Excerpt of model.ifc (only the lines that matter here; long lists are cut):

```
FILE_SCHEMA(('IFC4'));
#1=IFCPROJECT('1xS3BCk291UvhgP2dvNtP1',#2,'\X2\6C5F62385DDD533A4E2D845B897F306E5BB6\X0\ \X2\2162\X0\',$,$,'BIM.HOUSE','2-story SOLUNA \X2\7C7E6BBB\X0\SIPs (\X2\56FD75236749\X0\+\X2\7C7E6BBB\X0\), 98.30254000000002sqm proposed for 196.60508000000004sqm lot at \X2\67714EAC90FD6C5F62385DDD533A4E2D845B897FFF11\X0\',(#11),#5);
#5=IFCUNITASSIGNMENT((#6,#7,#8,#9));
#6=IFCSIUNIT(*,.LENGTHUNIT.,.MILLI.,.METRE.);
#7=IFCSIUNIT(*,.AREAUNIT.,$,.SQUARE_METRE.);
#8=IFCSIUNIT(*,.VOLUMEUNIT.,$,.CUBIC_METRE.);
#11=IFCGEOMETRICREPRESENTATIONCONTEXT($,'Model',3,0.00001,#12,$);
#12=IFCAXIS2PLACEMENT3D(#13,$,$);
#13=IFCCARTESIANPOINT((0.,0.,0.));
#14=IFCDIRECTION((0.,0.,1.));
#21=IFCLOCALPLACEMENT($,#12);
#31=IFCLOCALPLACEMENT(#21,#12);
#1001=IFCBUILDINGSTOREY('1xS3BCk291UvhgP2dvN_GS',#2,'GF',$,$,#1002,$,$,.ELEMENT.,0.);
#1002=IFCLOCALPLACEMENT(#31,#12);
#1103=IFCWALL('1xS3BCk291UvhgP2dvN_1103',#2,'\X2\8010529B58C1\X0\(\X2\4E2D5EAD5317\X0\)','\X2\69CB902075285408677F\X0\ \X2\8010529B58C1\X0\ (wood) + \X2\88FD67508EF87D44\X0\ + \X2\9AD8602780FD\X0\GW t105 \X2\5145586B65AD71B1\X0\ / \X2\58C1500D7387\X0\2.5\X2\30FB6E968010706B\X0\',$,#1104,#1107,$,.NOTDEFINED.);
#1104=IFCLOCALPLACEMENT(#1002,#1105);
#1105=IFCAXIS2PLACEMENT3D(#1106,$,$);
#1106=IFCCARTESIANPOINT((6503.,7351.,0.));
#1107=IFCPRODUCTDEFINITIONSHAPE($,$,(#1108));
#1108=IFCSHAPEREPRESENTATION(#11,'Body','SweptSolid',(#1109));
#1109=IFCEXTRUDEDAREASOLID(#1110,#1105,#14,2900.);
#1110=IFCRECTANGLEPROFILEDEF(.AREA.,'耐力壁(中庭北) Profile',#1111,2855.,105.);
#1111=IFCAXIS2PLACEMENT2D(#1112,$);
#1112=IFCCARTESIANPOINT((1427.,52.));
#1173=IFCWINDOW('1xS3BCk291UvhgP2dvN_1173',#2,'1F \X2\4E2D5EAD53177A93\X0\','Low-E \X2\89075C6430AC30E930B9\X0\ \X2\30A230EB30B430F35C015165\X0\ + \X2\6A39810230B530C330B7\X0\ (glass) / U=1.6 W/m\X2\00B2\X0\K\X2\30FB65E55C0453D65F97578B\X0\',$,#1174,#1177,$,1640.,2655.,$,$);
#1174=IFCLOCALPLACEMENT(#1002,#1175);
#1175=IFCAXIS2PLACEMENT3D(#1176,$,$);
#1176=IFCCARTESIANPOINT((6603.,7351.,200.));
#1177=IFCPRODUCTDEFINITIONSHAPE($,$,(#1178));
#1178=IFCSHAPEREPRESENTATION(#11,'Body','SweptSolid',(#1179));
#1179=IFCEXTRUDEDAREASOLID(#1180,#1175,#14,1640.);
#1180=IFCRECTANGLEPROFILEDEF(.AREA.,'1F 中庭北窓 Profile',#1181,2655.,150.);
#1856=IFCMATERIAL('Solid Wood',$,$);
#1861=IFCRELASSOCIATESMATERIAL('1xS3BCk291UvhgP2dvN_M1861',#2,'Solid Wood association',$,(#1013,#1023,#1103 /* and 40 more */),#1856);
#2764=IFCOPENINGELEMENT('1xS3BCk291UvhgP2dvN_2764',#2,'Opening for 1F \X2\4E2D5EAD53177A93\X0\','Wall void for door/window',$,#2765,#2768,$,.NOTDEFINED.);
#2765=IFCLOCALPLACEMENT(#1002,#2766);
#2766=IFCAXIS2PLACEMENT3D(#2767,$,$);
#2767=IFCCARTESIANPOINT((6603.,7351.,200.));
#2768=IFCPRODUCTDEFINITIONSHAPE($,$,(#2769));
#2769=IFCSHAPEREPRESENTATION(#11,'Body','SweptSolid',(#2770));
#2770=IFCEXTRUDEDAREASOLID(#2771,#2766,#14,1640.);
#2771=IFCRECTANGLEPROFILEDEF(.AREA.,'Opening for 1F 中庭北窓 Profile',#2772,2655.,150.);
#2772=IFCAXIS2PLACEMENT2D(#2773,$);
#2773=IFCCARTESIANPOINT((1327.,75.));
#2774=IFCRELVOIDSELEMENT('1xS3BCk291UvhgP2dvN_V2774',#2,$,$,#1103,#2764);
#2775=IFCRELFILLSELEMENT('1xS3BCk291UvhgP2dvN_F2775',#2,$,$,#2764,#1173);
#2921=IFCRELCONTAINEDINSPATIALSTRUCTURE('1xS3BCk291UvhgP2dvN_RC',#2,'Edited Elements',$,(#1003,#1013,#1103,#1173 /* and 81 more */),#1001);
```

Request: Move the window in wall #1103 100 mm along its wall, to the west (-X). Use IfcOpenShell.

```python
import ifcopenshell
import ifcopenshell.api.geometry
import ifcopenshell.util.placement
import ifcopenshell.util.unit

model = ifcopenshell.open("model.ifc")
unit_scale = ifcopenshell.util.unit.calculate_unit_scale(model)

window = model.by_id(1173)
opening = window.FillsVoids[0].RelatingOpeningElement
wall = opening.VoidsElements[0].RelatingBuildingElement

wall_matrix = ifcopenshell.util.placement.get_local_placement(wall.ObjectPlacement)
shift = wall_matrix[:3, 0] * -0.1 / unit_scale
before = ifcopenshell.util.placement.get_local_placement(window.ObjectPlacement)[:3, 3].copy()

# The window is not placed relative to its opening, so move both.
for product in (opening, window):
    matrix = ifcopenshell.util.placement.get_local_placement(product.ObjectPlacement)
    matrix[:3, 3] += shift
    ifcopenshell.api.geometry.edit_object_placement(model, product=product, matrix=matrix, is_si=False)

after = ifcopenshell.util.placement.get_local_placement(window.ObjectPlacement)[:3, 3]
print("window moved by", (after - before).round(3) + 0.0)

model.write("model_v2.ifc")
```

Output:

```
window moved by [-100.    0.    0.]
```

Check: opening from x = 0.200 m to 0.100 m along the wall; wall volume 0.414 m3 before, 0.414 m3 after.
